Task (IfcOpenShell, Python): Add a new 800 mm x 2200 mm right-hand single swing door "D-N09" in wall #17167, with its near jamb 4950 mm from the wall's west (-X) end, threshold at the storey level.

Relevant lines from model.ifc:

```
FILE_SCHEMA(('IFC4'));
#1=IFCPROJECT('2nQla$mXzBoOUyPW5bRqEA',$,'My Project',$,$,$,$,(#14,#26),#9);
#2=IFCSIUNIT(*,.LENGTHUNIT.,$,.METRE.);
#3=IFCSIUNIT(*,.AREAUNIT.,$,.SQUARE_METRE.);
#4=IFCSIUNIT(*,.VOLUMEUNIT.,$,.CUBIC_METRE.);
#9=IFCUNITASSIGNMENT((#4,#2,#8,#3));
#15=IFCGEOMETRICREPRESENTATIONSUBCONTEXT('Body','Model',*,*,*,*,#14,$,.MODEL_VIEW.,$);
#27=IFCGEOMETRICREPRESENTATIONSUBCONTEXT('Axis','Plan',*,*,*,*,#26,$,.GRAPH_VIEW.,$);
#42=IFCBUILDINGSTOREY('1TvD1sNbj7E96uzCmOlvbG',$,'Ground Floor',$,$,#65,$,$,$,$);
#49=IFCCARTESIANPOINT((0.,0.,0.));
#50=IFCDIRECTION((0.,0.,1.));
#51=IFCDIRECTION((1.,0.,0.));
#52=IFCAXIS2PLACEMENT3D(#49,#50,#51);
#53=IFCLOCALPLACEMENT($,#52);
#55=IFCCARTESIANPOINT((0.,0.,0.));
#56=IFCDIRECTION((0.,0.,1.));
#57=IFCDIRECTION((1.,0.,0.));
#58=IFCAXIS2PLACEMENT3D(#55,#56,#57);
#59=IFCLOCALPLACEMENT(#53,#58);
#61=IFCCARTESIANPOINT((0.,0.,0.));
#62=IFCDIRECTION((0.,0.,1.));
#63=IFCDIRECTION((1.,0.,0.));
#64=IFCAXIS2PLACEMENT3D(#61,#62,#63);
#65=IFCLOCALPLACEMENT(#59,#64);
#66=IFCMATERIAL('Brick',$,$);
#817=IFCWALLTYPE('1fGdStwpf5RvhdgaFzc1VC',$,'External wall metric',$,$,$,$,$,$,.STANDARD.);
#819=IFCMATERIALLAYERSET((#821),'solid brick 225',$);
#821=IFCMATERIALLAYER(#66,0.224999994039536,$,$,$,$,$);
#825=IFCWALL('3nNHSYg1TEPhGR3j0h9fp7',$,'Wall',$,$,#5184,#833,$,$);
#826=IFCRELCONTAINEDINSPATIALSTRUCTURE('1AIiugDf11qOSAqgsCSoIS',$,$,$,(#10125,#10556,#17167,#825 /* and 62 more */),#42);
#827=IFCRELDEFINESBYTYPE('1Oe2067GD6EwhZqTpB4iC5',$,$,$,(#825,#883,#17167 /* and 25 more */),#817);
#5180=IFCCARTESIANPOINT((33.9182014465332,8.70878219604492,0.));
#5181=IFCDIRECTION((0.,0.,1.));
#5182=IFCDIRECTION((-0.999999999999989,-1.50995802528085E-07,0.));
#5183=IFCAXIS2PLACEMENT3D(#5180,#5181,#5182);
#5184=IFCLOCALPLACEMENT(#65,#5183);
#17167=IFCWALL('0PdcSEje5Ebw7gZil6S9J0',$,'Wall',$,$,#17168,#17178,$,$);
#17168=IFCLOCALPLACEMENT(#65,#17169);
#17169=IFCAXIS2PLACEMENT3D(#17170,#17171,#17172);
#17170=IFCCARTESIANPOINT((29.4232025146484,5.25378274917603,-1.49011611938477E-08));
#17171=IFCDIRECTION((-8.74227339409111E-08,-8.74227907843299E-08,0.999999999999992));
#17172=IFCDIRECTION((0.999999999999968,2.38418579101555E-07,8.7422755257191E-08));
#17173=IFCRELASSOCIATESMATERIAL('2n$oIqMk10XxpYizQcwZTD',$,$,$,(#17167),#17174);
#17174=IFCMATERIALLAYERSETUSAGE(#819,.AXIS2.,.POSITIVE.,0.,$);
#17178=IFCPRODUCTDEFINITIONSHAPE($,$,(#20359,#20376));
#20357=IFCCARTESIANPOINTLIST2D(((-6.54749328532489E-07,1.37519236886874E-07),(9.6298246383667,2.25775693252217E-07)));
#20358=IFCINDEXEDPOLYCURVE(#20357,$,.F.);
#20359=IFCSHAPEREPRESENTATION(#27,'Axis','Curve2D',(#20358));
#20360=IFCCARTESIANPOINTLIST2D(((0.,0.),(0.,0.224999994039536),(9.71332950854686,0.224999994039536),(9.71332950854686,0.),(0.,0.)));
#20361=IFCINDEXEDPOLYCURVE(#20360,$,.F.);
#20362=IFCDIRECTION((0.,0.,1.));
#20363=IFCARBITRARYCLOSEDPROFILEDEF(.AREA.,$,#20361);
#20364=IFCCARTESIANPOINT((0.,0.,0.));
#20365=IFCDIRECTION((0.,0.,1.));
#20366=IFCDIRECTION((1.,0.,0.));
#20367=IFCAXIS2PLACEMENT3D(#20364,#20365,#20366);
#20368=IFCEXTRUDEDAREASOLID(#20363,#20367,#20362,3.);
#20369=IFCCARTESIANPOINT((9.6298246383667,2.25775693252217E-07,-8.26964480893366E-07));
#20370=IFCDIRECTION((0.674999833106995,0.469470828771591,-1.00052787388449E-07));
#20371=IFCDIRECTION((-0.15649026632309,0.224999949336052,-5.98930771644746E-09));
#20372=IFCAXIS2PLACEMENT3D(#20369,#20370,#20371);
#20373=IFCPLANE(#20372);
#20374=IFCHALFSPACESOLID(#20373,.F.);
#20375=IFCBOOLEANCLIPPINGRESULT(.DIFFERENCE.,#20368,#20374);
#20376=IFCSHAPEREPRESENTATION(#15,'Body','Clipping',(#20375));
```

```python
import numpy as np
import ifcopenshell
import ifcopenshell.api.feature
import ifcopenshell.api.geometry
import ifcopenshell.api.root
import ifcopenshell.api.spatial
import ifcopenshell.geom
import ifcopenshell.util.element
import ifcopenshell.util.placement
import ifcopenshell.util.representation
import ifcopenshell.util.shape
import ifcopenshell.util.unit

model = ifcopenshell.open("model.ifc")
unit_scale = ifcopenshell.util.unit.calculate_unit_scale(model)
settings = ifcopenshell.geom.settings()


def volume(element):
    """Net volume in cubic metres, openings subtracted."""
    shape = ifcopenshell.geom.create_shape(settings, element)
    return ifcopenshell.util.shape.get_volume(shape.geometry)


wall = model.by_guid("0PdcSEje5Ebw7gZil6S9J0")
storey = ifcopenshell.util.element.get_container(wall, ifc_class="IfcBuildingStorey")
context = ifcopenshell.util.representation.get_context(model, "Model", "Body", "MODEL_VIEW")
before = volume(wall)

width, height, from_end, sill = 0.8, 2.2, 4.95, 0.0  # metres

# The wall runs along its own X axis, and the end named is its -X end.
wall_shape = ifcopenshell.geom.create_shape(settings, wall)
x, y, z = ifcopenshell.util.shape.get_vertices(wall_shape.geometry).T
start = x.min() + from_end
face, thickness = float(y.min()), float(y.max() - y.min())
wall_matrix = ifcopenshell.util.placement.get_local_placement(wall.ObjectPlacement)
level = ifcopenshell.util.placement.get_local_placement(storey.ObjectPlacement)[2, 3]


def in_wall(x, y):
    """Placement at x, y metres in the wall's axes, at sill height."""
    matrix = wall_matrix.copy()
    matrix[:, 3] = wall_matrix @ np.array([x / unit_scale, y / unit_scale, 0.0, 1.0])
    matrix[2, 3] = level + sill / unit_scale
    return matrix


# Opening: a box that overshoots both wall faces by 50 mm.
opening = ifcopenshell.api.root.create_entity(model, ifc_class="IfcOpeningElement", predefined_type="OPENING")
box = ifcopenshell.api.geometry.add_wall_representation(
    model, context=context, length=width, height=height, thickness=thickness + 0.1
)
ifcopenshell.api.geometry.assign_representation(model, product=opening, representation=box)
ifcopenshell.api.geometry.edit_object_placement(model, product=opening, matrix=in_wall(start, face - 0.05), is_si=False)
ifcopenshell.api.feature.add_feature(model, feature=opening, element=wall)

door = ifcopenshell.api.root.create_entity(model, ifc_class="IfcDoor", name="D-N09", predefined_type="DOOR")
door.OverallWidth, door.OverallHeight = width / unit_scale, height / unit_scale
door.OperationType = "SINGLE_SWING_RIGHT"
body = ifcopenshell.api.geometry.add_door_representation(
    model,
    context=context,
    overall_width=door.OverallWidth,
    overall_height=door.OverallHeight,
    operation_type="SINGLE_SWING_RIGHT",
    lining_properties={"LiningDepth": thickness / unit_scale, "ThresholdDepth": thickness / unit_scale},
)
ifcopenshell.api.geometry.assign_representation(model, product=door, representation=body)
ifcopenshell.api.spatial.assign_container(model, products=[door], relating_structure=storey)
ifcopenshell.api.feature.add_filling(model, opening=opening, element=door)

# The lining spans the wall, so the door starts at the wall face.
ifcopenshell.api.geometry.edit_object_placement(model, product=door, matrix=in_wall(start, face), is_si=False)

after = volume(wall)

print(f"wall volume {before:.3f} -> {after:.3f} m3")

model.write("model_edited.ifc")
```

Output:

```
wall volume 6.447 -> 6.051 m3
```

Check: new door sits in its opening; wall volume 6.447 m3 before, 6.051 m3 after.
